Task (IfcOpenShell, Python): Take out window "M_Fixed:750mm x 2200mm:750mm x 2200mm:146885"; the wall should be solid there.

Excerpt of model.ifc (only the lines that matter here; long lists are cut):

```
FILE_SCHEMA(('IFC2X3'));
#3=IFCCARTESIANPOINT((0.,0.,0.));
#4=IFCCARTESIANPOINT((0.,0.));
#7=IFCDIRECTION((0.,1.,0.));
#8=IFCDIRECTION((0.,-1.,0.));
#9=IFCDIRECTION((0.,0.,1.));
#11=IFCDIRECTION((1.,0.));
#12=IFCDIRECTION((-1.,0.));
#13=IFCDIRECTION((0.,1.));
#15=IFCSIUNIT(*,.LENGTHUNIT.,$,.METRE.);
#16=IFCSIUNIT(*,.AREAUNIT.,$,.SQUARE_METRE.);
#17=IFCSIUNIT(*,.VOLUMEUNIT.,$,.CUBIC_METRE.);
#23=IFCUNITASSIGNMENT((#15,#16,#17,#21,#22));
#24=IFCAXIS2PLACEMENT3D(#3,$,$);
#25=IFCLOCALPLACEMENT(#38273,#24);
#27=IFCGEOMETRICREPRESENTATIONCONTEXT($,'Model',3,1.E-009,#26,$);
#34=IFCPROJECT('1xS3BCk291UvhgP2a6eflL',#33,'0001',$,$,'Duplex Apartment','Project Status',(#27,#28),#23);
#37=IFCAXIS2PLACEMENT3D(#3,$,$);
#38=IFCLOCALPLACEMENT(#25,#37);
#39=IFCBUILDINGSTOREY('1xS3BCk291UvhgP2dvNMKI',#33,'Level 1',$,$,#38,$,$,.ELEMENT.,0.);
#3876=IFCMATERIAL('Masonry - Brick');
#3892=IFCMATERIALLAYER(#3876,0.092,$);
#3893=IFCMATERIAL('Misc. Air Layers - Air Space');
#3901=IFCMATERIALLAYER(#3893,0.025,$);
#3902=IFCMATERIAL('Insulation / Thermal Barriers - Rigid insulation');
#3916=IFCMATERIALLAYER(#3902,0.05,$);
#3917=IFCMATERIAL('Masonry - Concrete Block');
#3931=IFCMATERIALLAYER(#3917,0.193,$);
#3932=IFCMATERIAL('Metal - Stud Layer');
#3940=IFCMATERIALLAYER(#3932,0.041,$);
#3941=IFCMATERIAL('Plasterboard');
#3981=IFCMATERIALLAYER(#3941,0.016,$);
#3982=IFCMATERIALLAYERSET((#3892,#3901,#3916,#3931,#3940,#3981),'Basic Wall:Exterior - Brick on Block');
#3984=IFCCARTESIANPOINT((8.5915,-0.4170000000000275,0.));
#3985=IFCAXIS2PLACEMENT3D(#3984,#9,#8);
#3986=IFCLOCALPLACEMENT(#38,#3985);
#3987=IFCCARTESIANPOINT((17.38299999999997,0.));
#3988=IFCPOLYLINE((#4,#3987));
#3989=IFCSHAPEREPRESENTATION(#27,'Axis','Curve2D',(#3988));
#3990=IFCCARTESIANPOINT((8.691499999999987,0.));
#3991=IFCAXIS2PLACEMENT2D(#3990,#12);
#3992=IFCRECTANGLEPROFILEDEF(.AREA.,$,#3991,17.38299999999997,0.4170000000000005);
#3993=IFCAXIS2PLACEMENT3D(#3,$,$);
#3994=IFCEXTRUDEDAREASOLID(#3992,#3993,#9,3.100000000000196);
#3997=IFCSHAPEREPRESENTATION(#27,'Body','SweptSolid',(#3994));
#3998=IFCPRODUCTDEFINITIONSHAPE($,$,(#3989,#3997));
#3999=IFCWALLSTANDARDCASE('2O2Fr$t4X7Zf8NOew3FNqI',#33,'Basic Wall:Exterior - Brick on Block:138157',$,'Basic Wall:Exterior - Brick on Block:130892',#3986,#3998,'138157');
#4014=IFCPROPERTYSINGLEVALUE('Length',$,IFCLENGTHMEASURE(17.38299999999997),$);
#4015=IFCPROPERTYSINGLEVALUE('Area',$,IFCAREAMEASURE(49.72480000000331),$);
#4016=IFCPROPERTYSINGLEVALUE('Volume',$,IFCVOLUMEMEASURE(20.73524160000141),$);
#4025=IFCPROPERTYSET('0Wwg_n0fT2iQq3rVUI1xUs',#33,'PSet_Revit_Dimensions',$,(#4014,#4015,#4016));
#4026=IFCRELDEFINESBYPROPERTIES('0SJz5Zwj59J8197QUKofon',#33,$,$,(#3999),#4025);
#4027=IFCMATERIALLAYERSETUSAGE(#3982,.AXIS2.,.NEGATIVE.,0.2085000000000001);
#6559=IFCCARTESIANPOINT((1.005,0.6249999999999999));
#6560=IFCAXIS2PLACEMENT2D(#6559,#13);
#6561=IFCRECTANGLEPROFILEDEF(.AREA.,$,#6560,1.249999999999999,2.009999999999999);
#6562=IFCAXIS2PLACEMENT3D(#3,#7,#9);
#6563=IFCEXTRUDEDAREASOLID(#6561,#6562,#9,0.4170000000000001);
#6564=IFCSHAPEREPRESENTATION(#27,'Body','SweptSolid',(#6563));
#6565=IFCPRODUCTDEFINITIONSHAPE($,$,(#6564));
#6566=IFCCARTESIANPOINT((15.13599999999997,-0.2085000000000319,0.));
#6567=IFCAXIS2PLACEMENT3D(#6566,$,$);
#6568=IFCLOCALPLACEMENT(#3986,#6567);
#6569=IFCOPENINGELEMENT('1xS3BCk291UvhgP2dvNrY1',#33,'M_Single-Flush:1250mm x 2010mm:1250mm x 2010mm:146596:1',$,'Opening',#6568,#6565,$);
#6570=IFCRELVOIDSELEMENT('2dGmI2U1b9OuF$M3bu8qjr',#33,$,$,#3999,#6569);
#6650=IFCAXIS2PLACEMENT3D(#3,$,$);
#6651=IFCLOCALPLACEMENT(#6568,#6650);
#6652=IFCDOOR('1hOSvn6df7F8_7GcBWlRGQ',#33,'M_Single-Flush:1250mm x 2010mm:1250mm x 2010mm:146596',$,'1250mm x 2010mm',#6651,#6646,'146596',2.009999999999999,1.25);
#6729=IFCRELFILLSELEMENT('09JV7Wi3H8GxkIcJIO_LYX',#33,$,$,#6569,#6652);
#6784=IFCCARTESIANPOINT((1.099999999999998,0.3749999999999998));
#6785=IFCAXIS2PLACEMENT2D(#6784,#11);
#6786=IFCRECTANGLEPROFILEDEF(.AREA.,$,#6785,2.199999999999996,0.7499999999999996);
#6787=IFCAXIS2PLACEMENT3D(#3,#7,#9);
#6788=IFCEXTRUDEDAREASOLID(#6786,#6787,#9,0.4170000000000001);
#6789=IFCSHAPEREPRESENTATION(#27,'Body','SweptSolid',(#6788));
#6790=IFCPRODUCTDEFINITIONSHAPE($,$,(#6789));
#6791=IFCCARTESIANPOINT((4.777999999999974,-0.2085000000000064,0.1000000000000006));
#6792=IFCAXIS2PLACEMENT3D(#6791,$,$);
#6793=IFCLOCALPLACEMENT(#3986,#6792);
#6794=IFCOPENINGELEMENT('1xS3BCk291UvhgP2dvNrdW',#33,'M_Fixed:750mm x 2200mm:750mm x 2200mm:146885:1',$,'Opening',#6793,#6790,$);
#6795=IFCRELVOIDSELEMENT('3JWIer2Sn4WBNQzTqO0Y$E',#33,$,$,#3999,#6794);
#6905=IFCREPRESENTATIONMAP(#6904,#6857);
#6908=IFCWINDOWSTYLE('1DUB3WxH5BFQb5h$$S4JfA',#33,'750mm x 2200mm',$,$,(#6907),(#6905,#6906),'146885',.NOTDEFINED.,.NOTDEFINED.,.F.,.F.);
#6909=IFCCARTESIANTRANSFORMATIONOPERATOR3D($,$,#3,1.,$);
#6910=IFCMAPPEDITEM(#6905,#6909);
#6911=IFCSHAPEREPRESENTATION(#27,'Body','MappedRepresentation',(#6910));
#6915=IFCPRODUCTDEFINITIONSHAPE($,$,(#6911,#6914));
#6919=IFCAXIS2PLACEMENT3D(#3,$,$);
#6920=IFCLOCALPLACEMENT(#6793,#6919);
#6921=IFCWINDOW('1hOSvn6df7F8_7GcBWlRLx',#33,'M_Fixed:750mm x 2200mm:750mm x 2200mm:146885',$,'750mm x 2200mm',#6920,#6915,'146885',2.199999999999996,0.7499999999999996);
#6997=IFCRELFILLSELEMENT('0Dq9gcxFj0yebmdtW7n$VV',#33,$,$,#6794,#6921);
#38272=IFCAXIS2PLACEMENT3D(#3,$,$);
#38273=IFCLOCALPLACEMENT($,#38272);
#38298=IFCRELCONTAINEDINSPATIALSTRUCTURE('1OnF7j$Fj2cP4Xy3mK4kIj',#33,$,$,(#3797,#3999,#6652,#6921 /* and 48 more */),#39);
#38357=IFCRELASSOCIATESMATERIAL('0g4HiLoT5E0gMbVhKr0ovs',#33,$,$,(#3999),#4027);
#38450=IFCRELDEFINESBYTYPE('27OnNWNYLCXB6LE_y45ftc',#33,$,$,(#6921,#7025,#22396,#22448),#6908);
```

```python
import ifcopenshell
import ifcopenshell.api.feature
import ifcopenshell.api.pset
import ifcopenshell.api.root
import ifcopenshell.geom
import ifcopenshell.util.element
import ifcopenshell.util.shape
import ifcopenshell.util.unit

model = ifcopenshell.open("model.ifc")
area_scale = ifcopenshell.util.unit.calculate_unit_scale(model, "AREAUNIT")
volume_scale = ifcopenshell.util.unit.calculate_unit_scale(model, "VOLUMEUNIT")
settings = ifcopenshell.geom.settings()


def volume(element):
    """Net volume in cubic metres, openings subtracted."""
    shape = ifcopenshell.geom.create_shape(settings, element)
    return ifcopenshell.util.shape.get_volume(shape.geometry)


window = model.by_guid("1hOSvn6df7F8_7GcBWlRLx")
opening = window.FillsVoids[0].RelatingOpeningElement
wall = opening.VoidsElements[0].RelatingBuildingElement
before = volume(wall)

ifcopenshell.api.root.remove_product(model, product=window)
ifcopenshell.api.feature.remove_feature(model, feature=opening)

after = volume(wall)
thickness = 0.417  # wall thickness in metres

# Update the wall's stored quantities.
pset = model.by_id(ifcopenshell.util.element.get_pset(wall, "PSet_Revit_Dimensions", should_inherit=False)["id"])
ifcopenshell.api.pset.edit_pset(model, pset=pset, properties={
    "Area": model.create_entity("IfcAreaMeasure", after / thickness / area_scale),
    "Volume": model.create_entity("IfcVolumeMeasure", after / volume_scale),
})

print(f"wall volume {before:.3f} -> {after:.3f} m3")

model.write("model_v2.ifc")
```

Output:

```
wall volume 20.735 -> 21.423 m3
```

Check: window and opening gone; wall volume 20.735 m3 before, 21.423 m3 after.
